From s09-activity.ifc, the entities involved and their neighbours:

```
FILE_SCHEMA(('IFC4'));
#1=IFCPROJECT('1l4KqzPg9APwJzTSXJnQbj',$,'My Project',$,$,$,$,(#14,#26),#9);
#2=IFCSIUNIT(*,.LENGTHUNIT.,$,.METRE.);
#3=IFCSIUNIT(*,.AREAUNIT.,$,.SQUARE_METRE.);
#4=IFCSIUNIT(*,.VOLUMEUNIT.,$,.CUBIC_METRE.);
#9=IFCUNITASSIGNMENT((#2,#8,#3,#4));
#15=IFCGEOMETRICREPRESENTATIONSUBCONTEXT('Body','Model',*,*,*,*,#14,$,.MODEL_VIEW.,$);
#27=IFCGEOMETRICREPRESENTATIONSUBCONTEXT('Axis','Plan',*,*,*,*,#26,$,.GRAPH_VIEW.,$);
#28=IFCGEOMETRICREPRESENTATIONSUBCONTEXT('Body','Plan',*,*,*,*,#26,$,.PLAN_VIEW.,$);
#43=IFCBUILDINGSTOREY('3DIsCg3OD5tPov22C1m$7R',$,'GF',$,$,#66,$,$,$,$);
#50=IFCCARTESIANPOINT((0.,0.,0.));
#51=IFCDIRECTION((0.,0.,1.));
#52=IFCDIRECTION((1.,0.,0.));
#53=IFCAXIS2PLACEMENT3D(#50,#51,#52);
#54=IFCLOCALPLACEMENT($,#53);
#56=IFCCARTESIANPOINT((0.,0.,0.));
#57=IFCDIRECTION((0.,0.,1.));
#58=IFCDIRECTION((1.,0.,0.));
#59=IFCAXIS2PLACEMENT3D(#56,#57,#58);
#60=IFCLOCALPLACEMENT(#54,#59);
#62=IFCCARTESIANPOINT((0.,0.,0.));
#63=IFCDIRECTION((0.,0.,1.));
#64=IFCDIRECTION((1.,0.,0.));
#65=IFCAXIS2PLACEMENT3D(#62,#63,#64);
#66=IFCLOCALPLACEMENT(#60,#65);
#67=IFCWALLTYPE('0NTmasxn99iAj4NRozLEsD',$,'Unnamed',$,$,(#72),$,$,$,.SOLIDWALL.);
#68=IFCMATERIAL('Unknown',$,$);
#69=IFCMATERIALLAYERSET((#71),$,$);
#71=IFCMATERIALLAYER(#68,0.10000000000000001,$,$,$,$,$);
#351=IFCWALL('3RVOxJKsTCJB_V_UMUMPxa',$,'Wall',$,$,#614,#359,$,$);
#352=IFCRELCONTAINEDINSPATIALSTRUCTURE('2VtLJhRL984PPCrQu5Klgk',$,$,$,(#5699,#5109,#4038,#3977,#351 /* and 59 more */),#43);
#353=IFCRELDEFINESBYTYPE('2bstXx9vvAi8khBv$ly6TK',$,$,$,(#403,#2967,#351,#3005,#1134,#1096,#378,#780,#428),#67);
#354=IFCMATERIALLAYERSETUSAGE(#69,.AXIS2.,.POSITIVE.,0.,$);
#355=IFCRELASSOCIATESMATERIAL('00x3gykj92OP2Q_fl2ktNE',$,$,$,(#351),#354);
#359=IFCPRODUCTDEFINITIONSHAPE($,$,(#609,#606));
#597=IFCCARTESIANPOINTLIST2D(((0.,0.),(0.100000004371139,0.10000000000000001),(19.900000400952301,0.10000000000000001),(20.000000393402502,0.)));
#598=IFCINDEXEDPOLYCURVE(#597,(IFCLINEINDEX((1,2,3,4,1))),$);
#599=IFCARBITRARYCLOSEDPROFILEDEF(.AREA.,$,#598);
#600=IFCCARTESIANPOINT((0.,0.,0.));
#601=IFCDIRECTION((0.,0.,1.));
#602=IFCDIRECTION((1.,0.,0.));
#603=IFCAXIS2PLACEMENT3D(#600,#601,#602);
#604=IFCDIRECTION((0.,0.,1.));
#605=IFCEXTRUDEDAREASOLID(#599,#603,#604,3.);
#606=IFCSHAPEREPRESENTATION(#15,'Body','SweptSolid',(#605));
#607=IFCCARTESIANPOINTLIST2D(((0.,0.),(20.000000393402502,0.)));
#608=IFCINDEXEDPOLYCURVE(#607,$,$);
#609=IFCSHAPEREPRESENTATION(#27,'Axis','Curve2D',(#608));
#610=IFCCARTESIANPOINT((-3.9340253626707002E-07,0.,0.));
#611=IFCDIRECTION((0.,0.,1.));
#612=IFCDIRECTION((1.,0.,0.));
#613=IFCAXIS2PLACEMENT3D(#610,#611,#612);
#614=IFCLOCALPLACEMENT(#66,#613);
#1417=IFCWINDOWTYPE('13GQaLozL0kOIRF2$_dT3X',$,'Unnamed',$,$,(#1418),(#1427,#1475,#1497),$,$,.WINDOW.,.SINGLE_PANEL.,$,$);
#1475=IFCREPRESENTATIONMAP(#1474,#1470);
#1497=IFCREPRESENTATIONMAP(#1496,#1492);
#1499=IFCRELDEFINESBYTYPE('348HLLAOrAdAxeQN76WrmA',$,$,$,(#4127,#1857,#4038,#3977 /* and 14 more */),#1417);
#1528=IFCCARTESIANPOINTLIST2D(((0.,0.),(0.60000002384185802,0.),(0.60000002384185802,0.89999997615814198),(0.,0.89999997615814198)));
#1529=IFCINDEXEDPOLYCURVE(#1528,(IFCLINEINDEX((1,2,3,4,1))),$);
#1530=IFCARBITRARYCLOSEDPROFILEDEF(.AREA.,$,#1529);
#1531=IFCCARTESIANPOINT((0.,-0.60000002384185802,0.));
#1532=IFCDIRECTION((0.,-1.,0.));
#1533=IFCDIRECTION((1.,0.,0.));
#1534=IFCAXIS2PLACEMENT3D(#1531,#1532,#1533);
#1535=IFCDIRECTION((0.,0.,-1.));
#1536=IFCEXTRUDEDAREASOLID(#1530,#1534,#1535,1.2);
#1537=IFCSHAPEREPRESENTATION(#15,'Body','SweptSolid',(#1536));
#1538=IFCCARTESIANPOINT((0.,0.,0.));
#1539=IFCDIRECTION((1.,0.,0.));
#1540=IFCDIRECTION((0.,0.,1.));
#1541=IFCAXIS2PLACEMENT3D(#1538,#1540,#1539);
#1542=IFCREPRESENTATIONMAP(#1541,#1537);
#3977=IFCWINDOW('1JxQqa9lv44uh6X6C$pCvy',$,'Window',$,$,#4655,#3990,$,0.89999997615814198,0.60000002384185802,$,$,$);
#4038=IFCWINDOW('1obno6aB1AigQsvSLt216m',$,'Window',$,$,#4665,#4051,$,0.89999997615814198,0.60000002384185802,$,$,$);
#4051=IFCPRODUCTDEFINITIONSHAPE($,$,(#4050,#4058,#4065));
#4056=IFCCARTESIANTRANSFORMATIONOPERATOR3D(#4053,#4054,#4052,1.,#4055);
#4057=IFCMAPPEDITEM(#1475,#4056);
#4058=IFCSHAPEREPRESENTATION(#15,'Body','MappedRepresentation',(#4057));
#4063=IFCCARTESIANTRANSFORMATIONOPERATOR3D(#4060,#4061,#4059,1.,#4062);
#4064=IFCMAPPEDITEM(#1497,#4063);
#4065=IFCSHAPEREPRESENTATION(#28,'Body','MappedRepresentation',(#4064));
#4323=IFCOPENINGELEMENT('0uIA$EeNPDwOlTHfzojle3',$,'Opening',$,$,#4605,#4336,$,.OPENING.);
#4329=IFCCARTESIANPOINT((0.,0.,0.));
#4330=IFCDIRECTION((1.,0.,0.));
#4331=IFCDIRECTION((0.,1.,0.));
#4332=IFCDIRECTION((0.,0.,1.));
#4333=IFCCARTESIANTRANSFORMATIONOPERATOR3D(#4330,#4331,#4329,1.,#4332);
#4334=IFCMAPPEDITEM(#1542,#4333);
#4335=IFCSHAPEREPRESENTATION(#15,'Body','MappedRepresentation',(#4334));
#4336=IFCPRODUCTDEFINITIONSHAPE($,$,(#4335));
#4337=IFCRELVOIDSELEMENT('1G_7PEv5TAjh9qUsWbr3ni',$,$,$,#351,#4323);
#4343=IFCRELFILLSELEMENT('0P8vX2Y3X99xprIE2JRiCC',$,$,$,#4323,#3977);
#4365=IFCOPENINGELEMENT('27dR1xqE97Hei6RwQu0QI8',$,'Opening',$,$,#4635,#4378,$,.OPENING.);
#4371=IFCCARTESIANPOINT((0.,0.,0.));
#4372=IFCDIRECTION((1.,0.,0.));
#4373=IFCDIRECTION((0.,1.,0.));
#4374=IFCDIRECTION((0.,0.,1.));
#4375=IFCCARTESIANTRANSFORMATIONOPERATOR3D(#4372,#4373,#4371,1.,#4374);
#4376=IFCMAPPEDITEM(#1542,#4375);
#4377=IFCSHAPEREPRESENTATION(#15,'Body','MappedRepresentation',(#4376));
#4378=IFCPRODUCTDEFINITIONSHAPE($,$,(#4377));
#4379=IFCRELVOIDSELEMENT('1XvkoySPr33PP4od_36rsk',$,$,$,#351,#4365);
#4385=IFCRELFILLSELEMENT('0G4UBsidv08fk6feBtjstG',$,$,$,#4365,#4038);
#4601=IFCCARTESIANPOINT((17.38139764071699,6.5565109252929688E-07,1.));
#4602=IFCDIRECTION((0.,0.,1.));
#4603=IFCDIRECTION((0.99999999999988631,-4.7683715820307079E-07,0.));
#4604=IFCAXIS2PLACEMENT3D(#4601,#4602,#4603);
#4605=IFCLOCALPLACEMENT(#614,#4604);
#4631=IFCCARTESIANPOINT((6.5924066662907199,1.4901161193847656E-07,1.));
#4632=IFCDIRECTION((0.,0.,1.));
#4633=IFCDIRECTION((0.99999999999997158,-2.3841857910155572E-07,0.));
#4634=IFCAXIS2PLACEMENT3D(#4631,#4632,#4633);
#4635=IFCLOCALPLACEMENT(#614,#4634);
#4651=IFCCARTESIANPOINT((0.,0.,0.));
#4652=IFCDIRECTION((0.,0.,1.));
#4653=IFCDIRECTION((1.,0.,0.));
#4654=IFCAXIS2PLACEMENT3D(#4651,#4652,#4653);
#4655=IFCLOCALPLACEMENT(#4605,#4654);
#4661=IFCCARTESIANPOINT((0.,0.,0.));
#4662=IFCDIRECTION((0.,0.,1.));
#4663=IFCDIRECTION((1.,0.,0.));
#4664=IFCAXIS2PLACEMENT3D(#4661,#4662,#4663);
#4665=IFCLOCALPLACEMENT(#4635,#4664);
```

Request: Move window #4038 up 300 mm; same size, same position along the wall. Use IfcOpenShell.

```python
import numpy as np
import ifcopenshell
import ifcopenshell.api.geometry
import ifcopenshell.util.placement
import ifcopenshell.util.unit

model = ifcopenshell.open("s09-activity.ifc")
unit_scale = ifcopenshell.util.unit.calculate_unit_scale(model)

window = model.by_guid("1obno6aB1AigQsvSLt216m")
opening = window.FillsVoids[0].RelatingOpeningElement
dz = 0.3 / unit_scale

shift = np.array([0.0, 0.0, dz])
# The window is placed relative to its opening, so it follows when the opening moves.
matrix = ifcopenshell.util.placement.get_local_placement(opening.ObjectPlacement)
matrix[:3, 3] += shift
ifcopenshell.api.geometry.edit_object_placement(
    model, product=opening, matrix=matrix, is_si=False, should_transform_children=True
)

print(f"moved by {dz * unit_scale:+.3f} m")

model.write("s09-activity_updated.ifc")
```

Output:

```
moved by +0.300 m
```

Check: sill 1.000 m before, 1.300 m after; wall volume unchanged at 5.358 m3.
